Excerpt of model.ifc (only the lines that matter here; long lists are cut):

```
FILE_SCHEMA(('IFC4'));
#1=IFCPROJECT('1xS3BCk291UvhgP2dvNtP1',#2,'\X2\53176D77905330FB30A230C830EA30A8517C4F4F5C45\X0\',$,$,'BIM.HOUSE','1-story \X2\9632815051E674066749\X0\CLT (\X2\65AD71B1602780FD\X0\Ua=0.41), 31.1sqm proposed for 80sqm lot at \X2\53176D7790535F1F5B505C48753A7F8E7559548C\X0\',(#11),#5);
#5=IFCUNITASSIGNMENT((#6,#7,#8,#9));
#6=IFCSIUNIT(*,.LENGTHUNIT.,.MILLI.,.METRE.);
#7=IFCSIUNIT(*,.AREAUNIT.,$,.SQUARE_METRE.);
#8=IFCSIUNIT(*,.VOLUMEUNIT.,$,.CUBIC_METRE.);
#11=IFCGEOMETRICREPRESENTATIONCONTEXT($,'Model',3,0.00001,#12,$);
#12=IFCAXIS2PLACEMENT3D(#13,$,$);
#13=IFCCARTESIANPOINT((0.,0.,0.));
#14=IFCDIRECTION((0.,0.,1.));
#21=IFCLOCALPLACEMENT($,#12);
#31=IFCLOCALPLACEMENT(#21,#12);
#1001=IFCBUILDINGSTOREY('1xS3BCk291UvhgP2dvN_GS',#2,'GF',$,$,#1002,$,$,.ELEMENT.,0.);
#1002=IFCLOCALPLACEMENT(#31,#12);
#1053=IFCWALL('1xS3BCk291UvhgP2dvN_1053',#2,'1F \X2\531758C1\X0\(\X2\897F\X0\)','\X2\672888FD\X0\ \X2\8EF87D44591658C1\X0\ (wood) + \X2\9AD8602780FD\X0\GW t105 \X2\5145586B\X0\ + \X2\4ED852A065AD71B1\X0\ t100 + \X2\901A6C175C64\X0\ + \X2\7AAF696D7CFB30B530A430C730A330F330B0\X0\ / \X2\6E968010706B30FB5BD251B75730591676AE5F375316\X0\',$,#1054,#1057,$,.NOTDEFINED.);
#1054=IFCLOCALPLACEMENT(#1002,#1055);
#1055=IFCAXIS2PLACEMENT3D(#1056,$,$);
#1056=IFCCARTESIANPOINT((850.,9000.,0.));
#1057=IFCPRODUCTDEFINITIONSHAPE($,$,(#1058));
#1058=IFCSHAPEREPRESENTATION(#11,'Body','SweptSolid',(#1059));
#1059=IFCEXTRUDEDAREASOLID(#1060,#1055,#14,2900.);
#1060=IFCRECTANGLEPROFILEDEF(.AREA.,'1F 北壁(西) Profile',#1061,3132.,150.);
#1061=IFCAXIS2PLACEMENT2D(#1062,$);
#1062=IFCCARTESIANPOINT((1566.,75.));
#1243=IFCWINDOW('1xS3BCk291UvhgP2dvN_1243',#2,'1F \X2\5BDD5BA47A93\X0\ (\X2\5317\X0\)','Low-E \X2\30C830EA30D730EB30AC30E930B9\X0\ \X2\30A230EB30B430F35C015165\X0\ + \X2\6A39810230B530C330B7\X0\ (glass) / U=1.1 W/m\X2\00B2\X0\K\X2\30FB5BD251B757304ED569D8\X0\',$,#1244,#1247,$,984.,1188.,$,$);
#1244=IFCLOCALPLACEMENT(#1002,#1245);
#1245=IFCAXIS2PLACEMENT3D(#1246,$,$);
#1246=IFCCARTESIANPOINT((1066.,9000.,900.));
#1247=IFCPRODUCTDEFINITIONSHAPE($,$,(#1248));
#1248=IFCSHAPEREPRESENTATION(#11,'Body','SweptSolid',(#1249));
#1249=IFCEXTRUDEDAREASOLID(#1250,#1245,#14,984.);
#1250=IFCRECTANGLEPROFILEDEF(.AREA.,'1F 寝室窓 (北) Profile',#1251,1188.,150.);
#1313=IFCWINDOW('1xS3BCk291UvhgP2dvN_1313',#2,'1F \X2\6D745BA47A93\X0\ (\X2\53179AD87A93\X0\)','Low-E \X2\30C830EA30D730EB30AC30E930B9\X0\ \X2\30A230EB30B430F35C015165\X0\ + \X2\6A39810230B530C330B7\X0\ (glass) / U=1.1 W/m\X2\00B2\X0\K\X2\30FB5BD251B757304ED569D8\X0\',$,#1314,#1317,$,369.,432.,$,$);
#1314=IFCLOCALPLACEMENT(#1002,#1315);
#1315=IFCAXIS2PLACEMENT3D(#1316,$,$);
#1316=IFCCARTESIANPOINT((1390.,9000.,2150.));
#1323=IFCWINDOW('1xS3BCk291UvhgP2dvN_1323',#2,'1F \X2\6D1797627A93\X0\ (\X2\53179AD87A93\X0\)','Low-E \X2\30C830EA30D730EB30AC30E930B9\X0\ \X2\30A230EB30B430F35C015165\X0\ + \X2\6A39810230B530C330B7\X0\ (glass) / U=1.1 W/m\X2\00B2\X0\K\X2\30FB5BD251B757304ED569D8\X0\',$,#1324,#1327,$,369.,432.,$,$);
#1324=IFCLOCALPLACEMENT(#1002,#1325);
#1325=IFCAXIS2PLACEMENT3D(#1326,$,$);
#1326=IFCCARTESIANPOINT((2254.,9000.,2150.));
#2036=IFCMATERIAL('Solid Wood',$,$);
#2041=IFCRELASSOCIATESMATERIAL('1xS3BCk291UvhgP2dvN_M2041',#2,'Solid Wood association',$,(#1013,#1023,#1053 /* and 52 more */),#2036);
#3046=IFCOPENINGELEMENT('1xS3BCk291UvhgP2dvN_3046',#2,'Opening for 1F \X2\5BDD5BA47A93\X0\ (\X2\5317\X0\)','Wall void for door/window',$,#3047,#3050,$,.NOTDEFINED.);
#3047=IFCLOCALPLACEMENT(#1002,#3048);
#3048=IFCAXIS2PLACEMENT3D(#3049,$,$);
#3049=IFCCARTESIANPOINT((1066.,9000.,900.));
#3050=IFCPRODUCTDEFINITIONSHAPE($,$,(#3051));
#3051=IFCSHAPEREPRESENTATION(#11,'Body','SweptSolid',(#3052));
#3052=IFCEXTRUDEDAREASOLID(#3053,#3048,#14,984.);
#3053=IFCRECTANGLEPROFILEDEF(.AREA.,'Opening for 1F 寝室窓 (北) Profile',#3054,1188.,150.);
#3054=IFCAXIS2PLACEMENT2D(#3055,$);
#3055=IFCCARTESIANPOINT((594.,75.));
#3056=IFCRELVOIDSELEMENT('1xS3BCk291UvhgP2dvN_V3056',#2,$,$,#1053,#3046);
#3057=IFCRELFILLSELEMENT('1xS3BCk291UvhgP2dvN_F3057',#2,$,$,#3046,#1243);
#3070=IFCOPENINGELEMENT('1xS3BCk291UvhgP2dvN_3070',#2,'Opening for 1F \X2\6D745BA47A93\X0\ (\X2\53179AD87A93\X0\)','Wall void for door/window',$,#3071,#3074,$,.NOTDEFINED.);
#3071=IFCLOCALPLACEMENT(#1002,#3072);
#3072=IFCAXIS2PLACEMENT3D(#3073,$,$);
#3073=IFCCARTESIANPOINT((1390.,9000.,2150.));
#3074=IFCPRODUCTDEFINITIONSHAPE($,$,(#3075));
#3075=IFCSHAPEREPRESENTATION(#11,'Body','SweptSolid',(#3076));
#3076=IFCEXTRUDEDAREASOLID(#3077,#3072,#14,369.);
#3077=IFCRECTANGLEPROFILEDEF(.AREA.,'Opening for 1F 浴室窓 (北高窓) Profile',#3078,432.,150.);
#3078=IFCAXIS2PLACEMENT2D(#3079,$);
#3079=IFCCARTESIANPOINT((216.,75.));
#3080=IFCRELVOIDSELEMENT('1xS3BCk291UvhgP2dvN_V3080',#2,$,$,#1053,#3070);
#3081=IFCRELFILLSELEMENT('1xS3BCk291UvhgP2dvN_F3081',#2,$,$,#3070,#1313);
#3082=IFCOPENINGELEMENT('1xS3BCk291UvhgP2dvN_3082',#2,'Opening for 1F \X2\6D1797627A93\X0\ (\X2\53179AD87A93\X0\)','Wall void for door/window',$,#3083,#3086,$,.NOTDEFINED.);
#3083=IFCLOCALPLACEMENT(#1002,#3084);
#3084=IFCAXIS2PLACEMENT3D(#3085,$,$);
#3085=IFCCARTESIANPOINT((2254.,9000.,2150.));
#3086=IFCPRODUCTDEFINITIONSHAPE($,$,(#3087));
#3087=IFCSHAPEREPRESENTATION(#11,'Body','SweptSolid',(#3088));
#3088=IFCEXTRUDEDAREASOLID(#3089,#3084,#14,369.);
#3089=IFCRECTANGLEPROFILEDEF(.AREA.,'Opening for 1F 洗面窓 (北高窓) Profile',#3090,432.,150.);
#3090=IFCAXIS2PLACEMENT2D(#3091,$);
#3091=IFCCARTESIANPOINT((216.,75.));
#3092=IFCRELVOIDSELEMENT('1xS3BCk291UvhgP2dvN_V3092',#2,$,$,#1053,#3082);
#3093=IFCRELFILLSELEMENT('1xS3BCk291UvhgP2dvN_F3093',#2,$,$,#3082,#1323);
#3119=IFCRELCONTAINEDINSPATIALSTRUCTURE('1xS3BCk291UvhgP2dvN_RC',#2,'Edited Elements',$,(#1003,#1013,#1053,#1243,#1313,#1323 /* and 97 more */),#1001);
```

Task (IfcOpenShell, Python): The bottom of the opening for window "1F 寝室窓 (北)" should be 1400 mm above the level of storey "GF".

```python
import numpy as np
import ifcopenshell
import ifcopenshell.api.geometry
import ifcopenshell.geom
import ifcopenshell.util.element
import ifcopenshell.util.placement
import ifcopenshell.util.shape
import ifcopenshell.util.unit

model = ifcopenshell.open("model.ifc")
unit_scale = ifcopenshell.util.unit.calculate_unit_scale(model)

window = model.by_guid("1xS3BCk291UvhgP2dvN_1243")
opening = window.FillsVoids[0].RelatingOpeningElement
storey = ifcopenshell.util.element.get_container(window, ifc_class="IfcBuildingStorey")
level = ifcopenshell.util.placement.get_local_placement(storey.ObjectPlacement)[2, 3]

# The opening's origin need not be at the sill, so measure its lowest point.
shape = ifcopenshell.geom.create_shape(ifcopenshell.geom.settings(), opening)
bottom = ifcopenshell.util.shape.get_shape_bottom_elevation(shape, shape.geometry) / unit_scale
dz = level + 1400.0 - bottom

shift = np.array([0.0, 0.0, dz])
# The window is not placed relative to its opening, so move both.
for product in (opening, window):
    matrix = ifcopenshell.util.placement.get_local_placement(product.ObjectPlacement)
    matrix[:3, 3] += shift
    ifcopenshell.api.geometry.edit_object_placement(model, product=product, matrix=matrix, is_si=False)

print(f"moved by {dz * unit_scale:+.3f} m")

model.write("model_updated.ifc")
```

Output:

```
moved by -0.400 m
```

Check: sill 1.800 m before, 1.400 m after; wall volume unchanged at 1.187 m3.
